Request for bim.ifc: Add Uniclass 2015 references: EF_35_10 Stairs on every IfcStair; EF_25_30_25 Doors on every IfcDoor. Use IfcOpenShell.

First a look at what the model holds.

```python
import ifcopenshell

model = ifcopenshell.open("bim.ifc")
print(model.schema)
print("classifications:", [c.Name for c in model.by_type("IfcClassification")])
for ifc_class in ("IfcDoor", "IfcRoof", "IfcStair", "IfcWall", "IfcWindow"):
    print(ifc_class, len(model.by_type(ifc_class)))
```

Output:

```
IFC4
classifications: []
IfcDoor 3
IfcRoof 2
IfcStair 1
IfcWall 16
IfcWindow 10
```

```python
import ifcopenshell
import ifcopenshell.api.classification

model = ifcopenshell.open("bim.ifc")

system = ifcopenshell.api.classification.add_classification(model, classification="Uniclass 2015")

codes = {
    "IfcStair": ("EF_35_10", "Stairs"),
    "IfcDoor": ("EF_25_30_25", "Doors"),
}
for ifc_class, (code, name) in codes.items():
    products = model.by_type(ifc_class)
    ifcopenshell.api.classification.add_reference(
        model, products=products, classification=system, identification=code, name=name
    )
    print(code, len(products))

model.write("bim_rev.ifc")
```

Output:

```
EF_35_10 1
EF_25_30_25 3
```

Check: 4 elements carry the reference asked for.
